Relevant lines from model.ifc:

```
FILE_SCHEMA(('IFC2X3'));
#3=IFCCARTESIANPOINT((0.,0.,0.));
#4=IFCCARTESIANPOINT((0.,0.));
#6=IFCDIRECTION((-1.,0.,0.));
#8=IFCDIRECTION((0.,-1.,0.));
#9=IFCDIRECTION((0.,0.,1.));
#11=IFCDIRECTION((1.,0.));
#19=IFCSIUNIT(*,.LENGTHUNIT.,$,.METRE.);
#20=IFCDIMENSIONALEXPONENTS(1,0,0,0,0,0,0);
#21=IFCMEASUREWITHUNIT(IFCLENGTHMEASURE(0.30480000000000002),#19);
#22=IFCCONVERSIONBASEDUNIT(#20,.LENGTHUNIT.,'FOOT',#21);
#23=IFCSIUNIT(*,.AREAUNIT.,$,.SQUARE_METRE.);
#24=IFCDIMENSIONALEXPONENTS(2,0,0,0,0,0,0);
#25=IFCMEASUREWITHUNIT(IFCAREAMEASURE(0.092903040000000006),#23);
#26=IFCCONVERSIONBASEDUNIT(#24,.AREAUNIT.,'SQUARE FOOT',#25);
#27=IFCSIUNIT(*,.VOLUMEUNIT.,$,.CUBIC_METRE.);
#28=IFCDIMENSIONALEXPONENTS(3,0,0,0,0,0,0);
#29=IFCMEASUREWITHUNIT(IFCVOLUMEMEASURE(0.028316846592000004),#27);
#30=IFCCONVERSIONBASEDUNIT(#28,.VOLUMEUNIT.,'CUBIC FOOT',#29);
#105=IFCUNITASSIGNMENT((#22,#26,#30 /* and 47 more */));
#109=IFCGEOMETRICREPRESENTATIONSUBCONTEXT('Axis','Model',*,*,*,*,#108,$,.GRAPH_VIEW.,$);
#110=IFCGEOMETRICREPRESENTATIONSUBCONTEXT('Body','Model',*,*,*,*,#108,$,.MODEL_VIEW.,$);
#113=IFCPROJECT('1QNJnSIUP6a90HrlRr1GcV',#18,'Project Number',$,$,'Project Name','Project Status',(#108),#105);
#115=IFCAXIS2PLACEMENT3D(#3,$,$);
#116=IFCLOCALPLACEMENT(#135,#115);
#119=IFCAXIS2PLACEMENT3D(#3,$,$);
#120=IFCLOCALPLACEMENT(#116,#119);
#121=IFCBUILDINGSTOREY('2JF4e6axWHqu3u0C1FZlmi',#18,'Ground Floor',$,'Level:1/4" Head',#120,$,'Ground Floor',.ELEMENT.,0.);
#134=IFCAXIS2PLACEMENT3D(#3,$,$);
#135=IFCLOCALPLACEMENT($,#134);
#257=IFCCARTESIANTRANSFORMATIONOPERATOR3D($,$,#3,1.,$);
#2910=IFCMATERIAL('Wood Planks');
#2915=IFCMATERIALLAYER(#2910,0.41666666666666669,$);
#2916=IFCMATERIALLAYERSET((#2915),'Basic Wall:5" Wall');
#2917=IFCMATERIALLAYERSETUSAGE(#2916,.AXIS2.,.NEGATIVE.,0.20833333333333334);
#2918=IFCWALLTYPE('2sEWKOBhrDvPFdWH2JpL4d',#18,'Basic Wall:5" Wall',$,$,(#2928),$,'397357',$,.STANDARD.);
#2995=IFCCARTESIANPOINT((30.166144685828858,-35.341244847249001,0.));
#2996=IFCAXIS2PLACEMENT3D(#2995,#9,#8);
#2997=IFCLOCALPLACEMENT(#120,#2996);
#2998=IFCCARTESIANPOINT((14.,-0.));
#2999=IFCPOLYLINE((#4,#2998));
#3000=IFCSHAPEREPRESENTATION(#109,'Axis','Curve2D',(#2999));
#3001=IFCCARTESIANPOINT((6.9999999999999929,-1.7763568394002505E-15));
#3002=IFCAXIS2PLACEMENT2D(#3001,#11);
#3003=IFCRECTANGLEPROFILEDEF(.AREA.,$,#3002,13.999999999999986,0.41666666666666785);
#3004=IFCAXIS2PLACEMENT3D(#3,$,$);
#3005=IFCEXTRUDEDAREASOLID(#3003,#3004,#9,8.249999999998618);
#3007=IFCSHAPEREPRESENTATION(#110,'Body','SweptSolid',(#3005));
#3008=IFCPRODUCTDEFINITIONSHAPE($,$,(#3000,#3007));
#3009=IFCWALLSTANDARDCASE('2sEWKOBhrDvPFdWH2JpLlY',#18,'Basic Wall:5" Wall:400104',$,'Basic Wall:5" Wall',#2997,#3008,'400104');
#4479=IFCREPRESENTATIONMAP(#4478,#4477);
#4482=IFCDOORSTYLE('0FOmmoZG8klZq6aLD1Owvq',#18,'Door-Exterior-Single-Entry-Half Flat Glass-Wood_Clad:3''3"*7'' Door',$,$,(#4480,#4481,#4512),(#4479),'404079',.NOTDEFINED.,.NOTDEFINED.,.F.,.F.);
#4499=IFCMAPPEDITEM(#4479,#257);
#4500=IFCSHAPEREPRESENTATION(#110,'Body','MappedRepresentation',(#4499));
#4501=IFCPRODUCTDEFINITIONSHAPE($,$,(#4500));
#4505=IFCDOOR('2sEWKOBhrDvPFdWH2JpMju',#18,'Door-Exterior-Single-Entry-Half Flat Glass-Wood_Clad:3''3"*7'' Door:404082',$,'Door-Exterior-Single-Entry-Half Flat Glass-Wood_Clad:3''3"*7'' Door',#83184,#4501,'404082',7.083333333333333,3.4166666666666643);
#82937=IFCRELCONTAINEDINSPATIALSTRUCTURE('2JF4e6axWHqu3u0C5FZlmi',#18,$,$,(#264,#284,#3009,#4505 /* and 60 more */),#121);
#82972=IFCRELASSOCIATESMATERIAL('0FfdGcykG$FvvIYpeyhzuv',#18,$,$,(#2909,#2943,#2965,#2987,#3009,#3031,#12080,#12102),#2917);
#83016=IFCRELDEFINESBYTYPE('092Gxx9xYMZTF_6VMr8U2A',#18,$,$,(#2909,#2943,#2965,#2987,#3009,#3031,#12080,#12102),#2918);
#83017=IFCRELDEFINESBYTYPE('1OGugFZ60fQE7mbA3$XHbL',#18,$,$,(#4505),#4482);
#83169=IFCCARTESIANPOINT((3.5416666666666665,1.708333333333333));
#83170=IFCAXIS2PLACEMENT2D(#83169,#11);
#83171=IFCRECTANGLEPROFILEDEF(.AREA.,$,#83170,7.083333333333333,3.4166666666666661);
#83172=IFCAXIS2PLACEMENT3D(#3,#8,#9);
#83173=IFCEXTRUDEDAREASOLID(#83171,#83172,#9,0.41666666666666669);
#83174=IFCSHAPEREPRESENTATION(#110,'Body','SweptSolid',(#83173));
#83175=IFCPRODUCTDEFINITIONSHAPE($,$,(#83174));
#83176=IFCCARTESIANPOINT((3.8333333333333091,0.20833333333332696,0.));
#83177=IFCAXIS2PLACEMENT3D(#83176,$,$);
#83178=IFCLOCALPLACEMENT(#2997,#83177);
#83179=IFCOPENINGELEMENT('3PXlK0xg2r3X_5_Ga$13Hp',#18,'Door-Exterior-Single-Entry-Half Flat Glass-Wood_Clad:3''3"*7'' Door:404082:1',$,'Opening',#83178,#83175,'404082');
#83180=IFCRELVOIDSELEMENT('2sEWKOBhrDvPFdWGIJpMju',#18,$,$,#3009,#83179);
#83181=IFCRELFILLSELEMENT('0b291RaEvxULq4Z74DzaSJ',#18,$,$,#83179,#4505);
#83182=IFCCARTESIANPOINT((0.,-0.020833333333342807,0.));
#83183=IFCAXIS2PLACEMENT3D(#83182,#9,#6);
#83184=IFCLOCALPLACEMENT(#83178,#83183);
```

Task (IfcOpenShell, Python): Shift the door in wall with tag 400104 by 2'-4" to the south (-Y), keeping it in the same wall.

```python
import ifcopenshell
import ifcopenshell.api.geometry
import ifcopenshell.util.placement
import ifcopenshell.util.unit

model = ifcopenshell.open("model.ifc")
unit_scale = ifcopenshell.util.unit.calculate_unit_scale(model)

door = model.by_guid("2sEWKOBhrDvPFdWH2JpMju")
opening = door.FillsVoids[0].RelatingOpeningElement
wall = opening.VoidsElements[0].RelatingBuildingElement

wall_matrix = ifcopenshell.util.placement.get_local_placement(wall.ObjectPlacement)
shift = wall_matrix[:3, 0] * 28 * 0.0254 / unit_scale
before = ifcopenshell.util.placement.get_local_placement(door.ObjectPlacement)[:3, 3].copy()

# The door is placed relative to its opening, so it follows when the opening moves.
matrix = ifcopenshell.util.placement.get_local_placement(opening.ObjectPlacement)
matrix[:3, 3] += shift
ifcopenshell.api.geometry.edit_object_placement(
    model, product=opening, matrix=matrix, is_si=False, should_transform_children=True
)

after = ifcopenshell.util.placement.get_local_placement(door.ObjectPlacement)[:3, 3]
print("door moved by", (after - before).round(3) + 0.0)

model.write("model_updated.ifc")
```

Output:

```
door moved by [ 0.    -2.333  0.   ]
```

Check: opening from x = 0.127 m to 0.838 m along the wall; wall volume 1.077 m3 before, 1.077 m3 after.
